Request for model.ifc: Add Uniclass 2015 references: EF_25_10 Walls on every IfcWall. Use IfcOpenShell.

First a look at what the model holds.

```python
import ifcopenshell

model = ifcopenshell.open("model.ifc")
print(model.schema)
print("classifications:", [c.Name for c in model.by_type("IfcClassification")])
for ifc_class in ("IfcDoor", "IfcRoof", "IfcStair", "IfcWall", "IfcWindow"):
    print(ifc_class, len(model.by_type(ifc_class)))
```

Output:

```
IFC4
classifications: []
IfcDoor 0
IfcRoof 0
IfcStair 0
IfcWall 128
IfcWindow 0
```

```python
import ifcopenshell
import ifcopenshell.api.classification

model = ifcopenshell.open("model.ifc")

system = ifcopenshell.api.classification.add_classification(model, classification="Uniclass 2015")

codes = {
    "IfcWall": ("EF_25_10", "Walls"),
}
for ifc_class, (code, name) in codes.items():
    products = model.by_type(ifc_class)
    ifcopenshell.api.classification.add_reference(
        model, products=products, classification=system, identification=code, name=name
    )
    print(code, len(products))

model.write("model_rev.ifc")
```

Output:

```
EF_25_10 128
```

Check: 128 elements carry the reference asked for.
